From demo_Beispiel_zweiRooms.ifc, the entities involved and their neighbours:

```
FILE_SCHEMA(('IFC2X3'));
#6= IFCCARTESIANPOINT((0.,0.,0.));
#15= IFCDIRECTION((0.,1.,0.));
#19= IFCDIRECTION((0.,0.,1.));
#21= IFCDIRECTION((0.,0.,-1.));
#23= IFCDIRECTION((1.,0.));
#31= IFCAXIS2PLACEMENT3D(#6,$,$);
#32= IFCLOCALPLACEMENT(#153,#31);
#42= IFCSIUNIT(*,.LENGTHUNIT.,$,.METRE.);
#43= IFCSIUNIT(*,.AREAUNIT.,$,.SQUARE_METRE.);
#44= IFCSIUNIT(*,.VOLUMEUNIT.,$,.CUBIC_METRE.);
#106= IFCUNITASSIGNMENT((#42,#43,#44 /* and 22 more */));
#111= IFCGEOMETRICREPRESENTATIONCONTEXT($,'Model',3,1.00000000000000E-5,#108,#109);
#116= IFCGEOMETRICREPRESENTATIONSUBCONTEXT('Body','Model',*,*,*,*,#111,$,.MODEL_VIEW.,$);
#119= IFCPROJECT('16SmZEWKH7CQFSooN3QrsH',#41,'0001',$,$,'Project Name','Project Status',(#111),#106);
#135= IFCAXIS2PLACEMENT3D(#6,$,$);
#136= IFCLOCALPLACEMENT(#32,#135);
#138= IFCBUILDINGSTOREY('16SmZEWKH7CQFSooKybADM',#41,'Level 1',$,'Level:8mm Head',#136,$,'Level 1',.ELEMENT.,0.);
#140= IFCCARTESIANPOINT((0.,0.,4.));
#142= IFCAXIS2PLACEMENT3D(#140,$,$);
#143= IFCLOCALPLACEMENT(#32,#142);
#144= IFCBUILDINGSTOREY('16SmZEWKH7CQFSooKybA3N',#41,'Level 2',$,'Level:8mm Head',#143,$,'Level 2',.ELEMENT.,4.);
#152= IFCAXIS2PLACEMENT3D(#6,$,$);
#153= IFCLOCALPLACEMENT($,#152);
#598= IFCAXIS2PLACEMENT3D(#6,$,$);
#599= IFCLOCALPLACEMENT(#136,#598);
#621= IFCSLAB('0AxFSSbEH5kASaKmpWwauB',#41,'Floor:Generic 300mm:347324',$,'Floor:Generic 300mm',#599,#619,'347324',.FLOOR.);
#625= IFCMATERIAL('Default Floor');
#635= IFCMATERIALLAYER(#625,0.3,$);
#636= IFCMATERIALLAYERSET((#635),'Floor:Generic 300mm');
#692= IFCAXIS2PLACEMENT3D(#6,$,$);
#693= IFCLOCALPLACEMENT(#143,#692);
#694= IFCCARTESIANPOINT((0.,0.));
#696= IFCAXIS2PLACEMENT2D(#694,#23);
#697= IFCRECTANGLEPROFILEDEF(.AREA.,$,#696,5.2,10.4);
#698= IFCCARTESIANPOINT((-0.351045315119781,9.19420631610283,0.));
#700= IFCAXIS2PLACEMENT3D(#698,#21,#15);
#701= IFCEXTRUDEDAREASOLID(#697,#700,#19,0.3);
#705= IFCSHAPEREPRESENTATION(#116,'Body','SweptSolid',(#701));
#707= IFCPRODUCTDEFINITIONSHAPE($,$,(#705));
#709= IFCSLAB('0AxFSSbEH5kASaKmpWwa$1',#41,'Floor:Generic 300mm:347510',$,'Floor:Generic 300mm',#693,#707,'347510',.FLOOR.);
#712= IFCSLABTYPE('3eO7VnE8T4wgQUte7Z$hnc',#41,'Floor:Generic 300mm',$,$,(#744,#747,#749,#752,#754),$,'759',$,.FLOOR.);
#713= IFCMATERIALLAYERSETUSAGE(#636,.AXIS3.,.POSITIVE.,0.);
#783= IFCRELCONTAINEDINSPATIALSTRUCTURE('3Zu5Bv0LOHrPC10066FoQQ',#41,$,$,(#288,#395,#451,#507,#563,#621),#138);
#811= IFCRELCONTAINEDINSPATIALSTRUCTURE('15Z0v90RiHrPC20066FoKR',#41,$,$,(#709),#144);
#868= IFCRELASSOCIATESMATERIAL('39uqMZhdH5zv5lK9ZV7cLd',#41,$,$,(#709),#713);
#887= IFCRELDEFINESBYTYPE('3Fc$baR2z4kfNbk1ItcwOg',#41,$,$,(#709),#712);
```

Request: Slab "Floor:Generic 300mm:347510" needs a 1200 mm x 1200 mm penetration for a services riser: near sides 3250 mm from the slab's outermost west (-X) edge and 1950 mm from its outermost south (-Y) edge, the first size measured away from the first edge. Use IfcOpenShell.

```python
import numpy as np
import ifcopenshell
import ifcopenshell.api.feature
import ifcopenshell.api.geometry
import ifcopenshell.api.root
import ifcopenshell.geom
import ifcopenshell.util.placement
import ifcopenshell.util.representation
import ifcopenshell.util.shape
import ifcopenshell.util.unit

model = ifcopenshell.open("demo_Beispiel_zweiRooms.ifc")
unit_scale = ifcopenshell.util.unit.calculate_unit_scale(model)
settings = ifcopenshell.geom.settings()


def volume(element):
    """Net volume in cubic metres, openings subtracted."""
    shape = ifcopenshell.geom.create_shape(settings, element)
    return ifcopenshell.util.shape.get_volume(shape.geometry)


slab = model.by_guid("0AxFSSbEH5kASaKmpWwa$1")
before = volume(slab)

# Extent in the slab's own axes, in metres. The edges named are its -X and -Y sides.
slab_shape = ifcopenshell.geom.create_shape(settings, slab)
vertices = ifcopenshell.util.shape.get_vertices(slab_shape.geometry)
x_min, y_min, bottom = vertices.min(axis=0)
top = vertices[:, 2].max()

opening = ifcopenshell.api.root.create_entity(model, ifc_class="IfcOpeningElement", name="Services riser opening")
context = ifcopenshell.util.representation.get_context(model, "Model", "Body", "MODEL_VIEW")
width, depth = 1.2, 1.2
outline = [(0.0, 0.0), (width, 0.0), (width, depth), (0.0, depth), (0.0, 0.0)]
# Overshoot both faces by 50 mm so the cut is clean.
shape = ifcopenshell.api.geometry.add_slab_representation(
    model, context=context, depth=top - bottom + 0.1, polyline=outline
)
ifcopenshell.api.geometry.assign_representation(model, product=opening, representation=shape)

matrix = ifcopenshell.util.placement.get_local_placement(slab.ObjectPlacement)
matrix[:, 3] = matrix @ np.append(np.array([x_min + 3.25, y_min + 1.95, bottom - 0.05]) / unit_scale, 1.0)
ifcopenshell.api.geometry.edit_object_placement(model, product=opening, matrix=matrix, is_si=False)
ifcopenshell.api.feature.add_feature(model, feature=opening, element=slab)

after = volume(slab)

print(f"slab volume {before:.3f} -> {after:.3f} m3")

model.write("demo_Beispiel_zweiRooms_rev.ifc")
```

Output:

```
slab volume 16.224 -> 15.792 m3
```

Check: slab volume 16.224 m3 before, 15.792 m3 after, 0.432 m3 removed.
